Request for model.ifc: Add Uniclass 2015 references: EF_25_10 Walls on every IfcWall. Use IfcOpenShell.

First a look at what the model holds.

```python
import ifcopenshell

model = ifcopenshell.open("model.ifc")
print(model.schema)
print("classifications:", [c.Name for c in model.by_type("IfcClassification")])
for ifc_class in ("IfcDoor", "IfcRoof", "IfcStair", "IfcWall", "IfcWindow"):
    print(ifc_class, len(model.by_type(ifc_class)))
```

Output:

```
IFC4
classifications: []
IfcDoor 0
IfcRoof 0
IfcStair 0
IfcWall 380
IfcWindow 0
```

```python
import ifcopenshell
import ifcopenshell.api.classification

model = ifcopenshell.open("model.ifc")

system = ifcopenshell.api.classification.add_classification(model, classification="Uniclass 2015")

codes = {
    "IfcWall": ("EF_25_10", "Walls"),
}
for ifc_class, (code, name) in codes.items():
    products = model.by_type(ifc_class)
    ifcopenshell.api.classification.add_reference(
        model, products=products, classification=system, identification=code, name=name
    )
    print(code, len(products))

model.write("model_updated.ifc")
```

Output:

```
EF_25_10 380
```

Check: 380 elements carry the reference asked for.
